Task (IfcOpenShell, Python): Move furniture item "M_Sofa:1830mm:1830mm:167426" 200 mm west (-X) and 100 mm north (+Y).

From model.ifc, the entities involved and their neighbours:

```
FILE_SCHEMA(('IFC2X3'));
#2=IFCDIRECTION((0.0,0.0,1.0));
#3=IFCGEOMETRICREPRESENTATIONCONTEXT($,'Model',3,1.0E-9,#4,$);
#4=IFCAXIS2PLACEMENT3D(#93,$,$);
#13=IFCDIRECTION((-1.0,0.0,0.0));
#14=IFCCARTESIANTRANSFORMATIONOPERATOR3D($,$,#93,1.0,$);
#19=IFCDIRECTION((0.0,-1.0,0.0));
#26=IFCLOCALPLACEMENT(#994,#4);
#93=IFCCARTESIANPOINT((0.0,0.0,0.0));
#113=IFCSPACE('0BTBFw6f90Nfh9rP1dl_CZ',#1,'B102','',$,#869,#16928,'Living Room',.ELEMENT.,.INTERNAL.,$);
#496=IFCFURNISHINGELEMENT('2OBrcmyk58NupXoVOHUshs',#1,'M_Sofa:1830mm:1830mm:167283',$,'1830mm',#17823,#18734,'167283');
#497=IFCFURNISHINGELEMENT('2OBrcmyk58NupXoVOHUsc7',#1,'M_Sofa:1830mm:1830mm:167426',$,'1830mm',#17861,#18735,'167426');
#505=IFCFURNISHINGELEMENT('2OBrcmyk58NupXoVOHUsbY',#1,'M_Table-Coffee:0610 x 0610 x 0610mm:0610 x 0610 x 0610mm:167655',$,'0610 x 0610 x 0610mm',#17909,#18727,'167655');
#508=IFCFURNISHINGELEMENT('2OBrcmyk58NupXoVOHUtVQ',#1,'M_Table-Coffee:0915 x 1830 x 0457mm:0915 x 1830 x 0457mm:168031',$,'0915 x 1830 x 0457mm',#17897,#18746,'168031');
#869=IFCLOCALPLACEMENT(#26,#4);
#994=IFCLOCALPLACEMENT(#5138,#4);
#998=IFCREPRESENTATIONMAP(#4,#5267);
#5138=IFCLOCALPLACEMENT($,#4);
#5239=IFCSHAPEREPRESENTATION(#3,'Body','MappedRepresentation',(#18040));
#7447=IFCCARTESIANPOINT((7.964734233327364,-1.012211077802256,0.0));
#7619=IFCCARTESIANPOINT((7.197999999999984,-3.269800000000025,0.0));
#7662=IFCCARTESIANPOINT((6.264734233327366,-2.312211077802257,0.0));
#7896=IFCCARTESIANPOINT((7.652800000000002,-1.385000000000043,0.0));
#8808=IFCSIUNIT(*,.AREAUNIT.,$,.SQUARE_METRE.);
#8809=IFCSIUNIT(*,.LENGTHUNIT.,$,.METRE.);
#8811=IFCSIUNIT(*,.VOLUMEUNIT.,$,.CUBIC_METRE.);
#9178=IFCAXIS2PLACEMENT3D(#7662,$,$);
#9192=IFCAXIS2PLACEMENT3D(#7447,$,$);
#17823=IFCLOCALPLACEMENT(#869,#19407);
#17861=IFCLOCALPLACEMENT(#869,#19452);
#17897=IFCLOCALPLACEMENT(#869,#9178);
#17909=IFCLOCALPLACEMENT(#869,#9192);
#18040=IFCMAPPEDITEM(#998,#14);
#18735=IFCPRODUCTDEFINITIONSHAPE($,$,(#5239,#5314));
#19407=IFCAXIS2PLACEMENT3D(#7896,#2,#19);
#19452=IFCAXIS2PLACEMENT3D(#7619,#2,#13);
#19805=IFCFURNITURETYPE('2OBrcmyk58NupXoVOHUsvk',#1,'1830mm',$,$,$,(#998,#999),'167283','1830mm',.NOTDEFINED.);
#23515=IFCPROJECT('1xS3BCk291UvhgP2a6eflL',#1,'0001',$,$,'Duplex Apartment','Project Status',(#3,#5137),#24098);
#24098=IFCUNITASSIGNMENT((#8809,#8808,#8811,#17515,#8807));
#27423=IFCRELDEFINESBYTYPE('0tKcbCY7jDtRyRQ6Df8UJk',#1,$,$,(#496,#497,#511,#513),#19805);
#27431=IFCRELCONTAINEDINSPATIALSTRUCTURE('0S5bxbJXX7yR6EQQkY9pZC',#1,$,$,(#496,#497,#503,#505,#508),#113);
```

```python
import ifcopenshell
import ifcopenshell.api.geometry
import ifcopenshell.util.placement
import ifcopenshell.util.unit

model = ifcopenshell.open("model.ifc")
unit_scale = ifcopenshell.util.unit.calculate_unit_scale(model)

item = model.by_guid("2OBrcmyk58NupXoVOHUsc7")
matrix = ifcopenshell.util.placement.get_local_placement(item.ObjectPlacement)
matrix[0, 3] -= 0.2 / unit_scale
matrix[1, 3] += 0.1 / unit_scale
ifcopenshell.api.geometry.edit_object_placement(model, product=item, matrix=matrix, is_si=False)

print(ifcopenshell.util.placement.get_local_placement(item.ObjectPlacement).round(3) + 0.0)

model.write("model_edited.ifc")
```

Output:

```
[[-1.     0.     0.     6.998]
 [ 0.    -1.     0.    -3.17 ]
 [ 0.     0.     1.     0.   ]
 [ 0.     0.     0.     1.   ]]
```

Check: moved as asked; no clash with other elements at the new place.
